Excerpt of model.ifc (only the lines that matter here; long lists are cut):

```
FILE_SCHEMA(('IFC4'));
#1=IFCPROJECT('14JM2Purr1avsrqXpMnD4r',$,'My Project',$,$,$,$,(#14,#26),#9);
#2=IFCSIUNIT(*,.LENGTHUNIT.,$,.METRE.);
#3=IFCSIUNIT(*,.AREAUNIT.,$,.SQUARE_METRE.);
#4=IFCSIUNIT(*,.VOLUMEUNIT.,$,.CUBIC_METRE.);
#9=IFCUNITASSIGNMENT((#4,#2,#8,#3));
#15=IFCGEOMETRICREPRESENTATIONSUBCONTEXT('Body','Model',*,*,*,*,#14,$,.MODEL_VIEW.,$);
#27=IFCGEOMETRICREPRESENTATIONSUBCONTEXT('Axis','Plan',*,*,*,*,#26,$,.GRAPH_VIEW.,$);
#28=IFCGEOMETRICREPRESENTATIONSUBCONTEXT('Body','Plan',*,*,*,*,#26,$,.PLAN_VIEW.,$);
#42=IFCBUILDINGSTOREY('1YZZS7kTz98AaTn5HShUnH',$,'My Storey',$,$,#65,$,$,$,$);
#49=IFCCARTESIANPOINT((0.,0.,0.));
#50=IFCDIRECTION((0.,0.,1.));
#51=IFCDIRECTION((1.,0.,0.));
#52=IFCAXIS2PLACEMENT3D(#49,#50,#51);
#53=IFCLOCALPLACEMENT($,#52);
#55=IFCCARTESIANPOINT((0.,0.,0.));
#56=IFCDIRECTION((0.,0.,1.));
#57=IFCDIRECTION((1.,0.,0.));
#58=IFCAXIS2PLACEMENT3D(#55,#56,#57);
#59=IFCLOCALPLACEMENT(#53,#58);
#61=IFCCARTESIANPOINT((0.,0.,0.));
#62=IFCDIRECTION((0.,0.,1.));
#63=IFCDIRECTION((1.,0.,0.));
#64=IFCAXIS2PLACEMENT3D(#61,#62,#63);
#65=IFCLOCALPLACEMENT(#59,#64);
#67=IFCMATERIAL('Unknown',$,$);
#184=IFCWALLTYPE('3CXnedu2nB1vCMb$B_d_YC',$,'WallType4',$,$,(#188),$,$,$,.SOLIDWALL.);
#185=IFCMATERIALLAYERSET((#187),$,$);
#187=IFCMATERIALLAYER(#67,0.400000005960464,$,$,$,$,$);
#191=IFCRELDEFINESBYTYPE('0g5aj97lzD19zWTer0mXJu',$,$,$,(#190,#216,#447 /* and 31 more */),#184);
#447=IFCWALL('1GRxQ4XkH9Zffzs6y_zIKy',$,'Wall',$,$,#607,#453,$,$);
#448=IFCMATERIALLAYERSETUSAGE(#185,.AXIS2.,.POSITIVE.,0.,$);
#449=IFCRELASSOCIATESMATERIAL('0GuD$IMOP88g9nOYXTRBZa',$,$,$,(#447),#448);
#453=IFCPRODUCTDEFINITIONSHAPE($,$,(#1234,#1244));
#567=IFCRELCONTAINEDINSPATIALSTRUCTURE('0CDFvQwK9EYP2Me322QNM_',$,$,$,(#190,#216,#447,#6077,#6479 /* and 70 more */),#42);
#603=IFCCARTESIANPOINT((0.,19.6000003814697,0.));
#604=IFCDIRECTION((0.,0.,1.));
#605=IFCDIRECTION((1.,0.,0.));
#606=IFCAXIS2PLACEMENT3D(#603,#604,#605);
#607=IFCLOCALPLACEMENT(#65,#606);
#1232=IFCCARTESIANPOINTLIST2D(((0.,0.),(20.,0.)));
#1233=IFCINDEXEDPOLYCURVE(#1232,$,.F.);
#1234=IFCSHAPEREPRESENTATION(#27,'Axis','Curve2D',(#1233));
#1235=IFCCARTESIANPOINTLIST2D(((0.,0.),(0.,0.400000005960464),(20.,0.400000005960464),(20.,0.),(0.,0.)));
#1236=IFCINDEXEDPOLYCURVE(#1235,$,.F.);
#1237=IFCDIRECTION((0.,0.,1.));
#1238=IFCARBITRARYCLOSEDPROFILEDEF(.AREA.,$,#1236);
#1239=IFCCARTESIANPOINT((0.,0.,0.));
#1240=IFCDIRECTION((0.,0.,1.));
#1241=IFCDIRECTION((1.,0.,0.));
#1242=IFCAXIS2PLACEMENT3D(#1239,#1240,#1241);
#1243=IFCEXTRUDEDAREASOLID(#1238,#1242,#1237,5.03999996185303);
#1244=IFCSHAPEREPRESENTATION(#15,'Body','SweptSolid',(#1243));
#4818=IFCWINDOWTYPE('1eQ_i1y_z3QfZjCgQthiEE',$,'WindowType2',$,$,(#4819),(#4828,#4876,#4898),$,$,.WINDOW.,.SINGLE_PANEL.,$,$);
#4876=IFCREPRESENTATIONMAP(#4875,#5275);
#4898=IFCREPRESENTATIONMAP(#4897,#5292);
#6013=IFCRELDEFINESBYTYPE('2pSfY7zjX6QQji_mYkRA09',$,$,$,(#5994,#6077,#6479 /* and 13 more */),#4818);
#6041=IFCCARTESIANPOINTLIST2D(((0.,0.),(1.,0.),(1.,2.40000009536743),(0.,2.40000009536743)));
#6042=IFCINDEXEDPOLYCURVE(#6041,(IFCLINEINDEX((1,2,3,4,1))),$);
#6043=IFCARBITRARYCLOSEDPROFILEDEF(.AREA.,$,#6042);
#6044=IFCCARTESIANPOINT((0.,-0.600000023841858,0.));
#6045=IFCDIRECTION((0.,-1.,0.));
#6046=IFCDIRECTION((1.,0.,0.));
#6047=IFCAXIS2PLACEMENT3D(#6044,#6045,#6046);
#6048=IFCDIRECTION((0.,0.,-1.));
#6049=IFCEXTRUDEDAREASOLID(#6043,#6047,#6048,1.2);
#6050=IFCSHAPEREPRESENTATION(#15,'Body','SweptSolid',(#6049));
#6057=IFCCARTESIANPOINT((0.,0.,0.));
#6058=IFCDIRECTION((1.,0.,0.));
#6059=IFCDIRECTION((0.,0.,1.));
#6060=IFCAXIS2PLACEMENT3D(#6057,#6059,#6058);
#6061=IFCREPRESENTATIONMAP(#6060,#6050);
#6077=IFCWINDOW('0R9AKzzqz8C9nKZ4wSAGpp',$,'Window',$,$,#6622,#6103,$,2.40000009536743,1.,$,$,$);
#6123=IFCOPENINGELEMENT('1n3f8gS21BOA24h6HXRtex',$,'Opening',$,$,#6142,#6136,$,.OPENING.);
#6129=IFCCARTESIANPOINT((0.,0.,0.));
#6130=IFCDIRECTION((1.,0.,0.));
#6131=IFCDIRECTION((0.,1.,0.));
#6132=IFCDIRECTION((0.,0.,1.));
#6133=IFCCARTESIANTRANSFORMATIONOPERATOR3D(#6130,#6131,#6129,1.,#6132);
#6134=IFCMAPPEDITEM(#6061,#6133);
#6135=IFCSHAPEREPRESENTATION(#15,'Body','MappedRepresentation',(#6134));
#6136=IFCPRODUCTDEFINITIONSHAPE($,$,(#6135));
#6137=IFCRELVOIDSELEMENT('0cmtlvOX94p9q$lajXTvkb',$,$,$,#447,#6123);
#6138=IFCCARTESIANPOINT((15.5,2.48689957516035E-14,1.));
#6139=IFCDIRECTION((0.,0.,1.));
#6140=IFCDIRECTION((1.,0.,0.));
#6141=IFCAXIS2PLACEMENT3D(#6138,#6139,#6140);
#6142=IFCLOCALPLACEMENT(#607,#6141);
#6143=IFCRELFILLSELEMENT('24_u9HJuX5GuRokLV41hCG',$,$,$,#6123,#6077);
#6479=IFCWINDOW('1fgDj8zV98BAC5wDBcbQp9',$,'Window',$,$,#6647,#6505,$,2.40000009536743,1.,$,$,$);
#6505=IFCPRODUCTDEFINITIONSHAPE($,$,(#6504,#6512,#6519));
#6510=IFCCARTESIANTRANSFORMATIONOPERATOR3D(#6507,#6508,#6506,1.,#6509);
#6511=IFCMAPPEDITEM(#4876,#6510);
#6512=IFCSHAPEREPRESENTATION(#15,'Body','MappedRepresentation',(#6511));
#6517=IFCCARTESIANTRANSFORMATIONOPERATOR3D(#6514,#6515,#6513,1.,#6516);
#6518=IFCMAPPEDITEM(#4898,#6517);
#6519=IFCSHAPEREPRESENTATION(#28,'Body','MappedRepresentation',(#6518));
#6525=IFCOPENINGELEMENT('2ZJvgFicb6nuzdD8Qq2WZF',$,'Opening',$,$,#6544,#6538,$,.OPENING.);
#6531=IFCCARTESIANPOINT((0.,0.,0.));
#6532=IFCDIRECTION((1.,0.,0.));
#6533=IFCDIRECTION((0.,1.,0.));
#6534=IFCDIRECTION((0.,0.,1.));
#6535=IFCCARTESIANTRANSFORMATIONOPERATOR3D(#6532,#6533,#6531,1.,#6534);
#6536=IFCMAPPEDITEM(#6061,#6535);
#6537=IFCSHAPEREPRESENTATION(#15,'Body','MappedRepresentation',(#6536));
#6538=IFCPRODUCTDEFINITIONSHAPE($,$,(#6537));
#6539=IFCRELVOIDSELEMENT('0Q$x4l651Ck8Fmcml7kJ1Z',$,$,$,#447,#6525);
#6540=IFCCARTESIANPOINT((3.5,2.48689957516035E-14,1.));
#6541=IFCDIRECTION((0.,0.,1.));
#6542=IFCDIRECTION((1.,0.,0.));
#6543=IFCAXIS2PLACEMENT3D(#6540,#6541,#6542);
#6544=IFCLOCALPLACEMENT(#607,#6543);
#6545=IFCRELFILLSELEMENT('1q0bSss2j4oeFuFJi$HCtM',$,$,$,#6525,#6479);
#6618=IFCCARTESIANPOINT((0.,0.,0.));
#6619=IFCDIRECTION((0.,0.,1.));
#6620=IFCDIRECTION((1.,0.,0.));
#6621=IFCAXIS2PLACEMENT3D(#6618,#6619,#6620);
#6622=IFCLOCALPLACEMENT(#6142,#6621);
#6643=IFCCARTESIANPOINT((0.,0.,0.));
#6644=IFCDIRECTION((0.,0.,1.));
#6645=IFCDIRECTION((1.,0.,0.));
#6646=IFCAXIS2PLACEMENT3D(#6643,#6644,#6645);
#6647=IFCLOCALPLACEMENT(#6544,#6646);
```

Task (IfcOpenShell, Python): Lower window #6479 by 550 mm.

```python
import numpy as np
import ifcopenshell
import ifcopenshell.api.geometry
import ifcopenshell.util.placement
import ifcopenshell.util.unit

model = ifcopenshell.open("model.ifc")
unit_scale = ifcopenshell.util.unit.calculate_unit_scale(model)

window = model.by_guid("1fgDj8zV98BAC5wDBcbQp9")
opening = window.FillsVoids[0].RelatingOpeningElement
dz = -0.55 / unit_scale

shift = np.array([0.0, 0.0, dz])
# The window is placed relative to its opening, so it follows when the opening moves.
matrix = ifcopenshell.util.placement.get_local_placement(opening.ObjectPlacement)
matrix[:3, 3] += shift
ifcopenshell.api.geometry.edit_object_placement(
    model, product=opening, matrix=matrix, is_si=False, should_transform_children=True
)

print(f"moved by {dz * unit_scale:+.3f} m")

model.write("model_edited.ifc")
```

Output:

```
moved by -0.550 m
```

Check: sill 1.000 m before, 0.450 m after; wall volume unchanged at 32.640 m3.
